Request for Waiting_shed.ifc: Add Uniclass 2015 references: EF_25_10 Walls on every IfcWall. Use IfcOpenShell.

First a look at what the model holds.

```python
import ifcopenshell

model = ifcopenshell.open("Waiting_shed.ifc")
print(model.schema)
print("classifications:", [c.Name for c in model.by_type("IfcClassification")])
for ifc_class in ("IfcDoor", "IfcRoof", "IfcStair", "IfcWall", "IfcWindow"):
    print(ifc_class, len(model.by_type(ifc_class)))
```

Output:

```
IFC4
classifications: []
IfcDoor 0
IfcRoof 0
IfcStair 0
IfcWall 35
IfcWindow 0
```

```python
import ifcopenshell
import ifcopenshell.api.classification

model = ifcopenshell.open("Waiting_shed.ifc")

system = ifcopenshell.api.classification.add_classification(model, classification="Uniclass 2015")

codes = {
    "IfcWall": ("EF_25_10", "Walls"),
}
for ifc_class, (code, name) in codes.items():
    products = model.by_type(ifc_class)
    ifcopenshell.api.classification.add_reference(
        model, products=products, classification=system, identification=code, name=name
    )
    print(code, len(products))

model.write("Waiting_shed_edited.ifc")
```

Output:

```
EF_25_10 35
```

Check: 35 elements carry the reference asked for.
